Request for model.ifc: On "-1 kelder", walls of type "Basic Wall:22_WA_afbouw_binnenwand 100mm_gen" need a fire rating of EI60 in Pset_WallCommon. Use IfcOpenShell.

First a look at what the model holds.

```python
import ifcopenshell
import ifcopenshell.util.element

model = ifcopenshell.open("model.ifc")
print(model.schema)
storey = next(s for s in model.by_type("IfcBuildingStorey") if s.Name == "-1 kelder")
walls = [e for e in ifcopenshell.util.element.get_decomposition(storey) if e.is_a("IfcWall")]
seen = {}
for e in walls:
    element_type = ifcopenshell.util.element.get_type(e)
    key = (element_type.Name if element_type != e and element_type else None, ifcopenshell.util.element.get_pset(e, "Pset_WallCommon", "FireRating"))
    seen[key] = seen.get(key, 0) + 1
for (name, value), count in sorted(seen.items(), key=str):
    print(count, "x", name, "|", value)
```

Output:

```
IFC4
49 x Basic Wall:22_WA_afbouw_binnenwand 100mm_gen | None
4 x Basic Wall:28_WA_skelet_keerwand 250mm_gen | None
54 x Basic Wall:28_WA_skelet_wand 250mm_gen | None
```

```python
import ifcopenshell
import ifcopenshell.api.pset
import ifcopenshell.util.element

model = ifcopenshell.open("model.ifc")

storey = next(s for s in model.by_type("IfcBuildingStorey") if s.Name == "-1 kelder")
walls = [e for e in ifcopenshell.util.element.get_decomposition(storey) if e.is_a("IfcWall")]

count = 0
for e in walls:
    element_type = ifcopenshell.util.element.get_type(e)
    if element_type in (None, e) or element_type.Name != "Basic Wall:22_WA_afbouw_binnenwand 100mm_gen":
        continue
    # add_pset returns the element's existing set when there is one.
    pset = ifcopenshell.api.pset.add_pset(model, product=e, name="Pset_WallCommon")
    ifcopenshell.api.pset.edit_pset(model, pset=pset, properties={"FireRating": "EI60"})
    count += 1

print(count, "walls updated")

model.write("model_edited.ifc")
```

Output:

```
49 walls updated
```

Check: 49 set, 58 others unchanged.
